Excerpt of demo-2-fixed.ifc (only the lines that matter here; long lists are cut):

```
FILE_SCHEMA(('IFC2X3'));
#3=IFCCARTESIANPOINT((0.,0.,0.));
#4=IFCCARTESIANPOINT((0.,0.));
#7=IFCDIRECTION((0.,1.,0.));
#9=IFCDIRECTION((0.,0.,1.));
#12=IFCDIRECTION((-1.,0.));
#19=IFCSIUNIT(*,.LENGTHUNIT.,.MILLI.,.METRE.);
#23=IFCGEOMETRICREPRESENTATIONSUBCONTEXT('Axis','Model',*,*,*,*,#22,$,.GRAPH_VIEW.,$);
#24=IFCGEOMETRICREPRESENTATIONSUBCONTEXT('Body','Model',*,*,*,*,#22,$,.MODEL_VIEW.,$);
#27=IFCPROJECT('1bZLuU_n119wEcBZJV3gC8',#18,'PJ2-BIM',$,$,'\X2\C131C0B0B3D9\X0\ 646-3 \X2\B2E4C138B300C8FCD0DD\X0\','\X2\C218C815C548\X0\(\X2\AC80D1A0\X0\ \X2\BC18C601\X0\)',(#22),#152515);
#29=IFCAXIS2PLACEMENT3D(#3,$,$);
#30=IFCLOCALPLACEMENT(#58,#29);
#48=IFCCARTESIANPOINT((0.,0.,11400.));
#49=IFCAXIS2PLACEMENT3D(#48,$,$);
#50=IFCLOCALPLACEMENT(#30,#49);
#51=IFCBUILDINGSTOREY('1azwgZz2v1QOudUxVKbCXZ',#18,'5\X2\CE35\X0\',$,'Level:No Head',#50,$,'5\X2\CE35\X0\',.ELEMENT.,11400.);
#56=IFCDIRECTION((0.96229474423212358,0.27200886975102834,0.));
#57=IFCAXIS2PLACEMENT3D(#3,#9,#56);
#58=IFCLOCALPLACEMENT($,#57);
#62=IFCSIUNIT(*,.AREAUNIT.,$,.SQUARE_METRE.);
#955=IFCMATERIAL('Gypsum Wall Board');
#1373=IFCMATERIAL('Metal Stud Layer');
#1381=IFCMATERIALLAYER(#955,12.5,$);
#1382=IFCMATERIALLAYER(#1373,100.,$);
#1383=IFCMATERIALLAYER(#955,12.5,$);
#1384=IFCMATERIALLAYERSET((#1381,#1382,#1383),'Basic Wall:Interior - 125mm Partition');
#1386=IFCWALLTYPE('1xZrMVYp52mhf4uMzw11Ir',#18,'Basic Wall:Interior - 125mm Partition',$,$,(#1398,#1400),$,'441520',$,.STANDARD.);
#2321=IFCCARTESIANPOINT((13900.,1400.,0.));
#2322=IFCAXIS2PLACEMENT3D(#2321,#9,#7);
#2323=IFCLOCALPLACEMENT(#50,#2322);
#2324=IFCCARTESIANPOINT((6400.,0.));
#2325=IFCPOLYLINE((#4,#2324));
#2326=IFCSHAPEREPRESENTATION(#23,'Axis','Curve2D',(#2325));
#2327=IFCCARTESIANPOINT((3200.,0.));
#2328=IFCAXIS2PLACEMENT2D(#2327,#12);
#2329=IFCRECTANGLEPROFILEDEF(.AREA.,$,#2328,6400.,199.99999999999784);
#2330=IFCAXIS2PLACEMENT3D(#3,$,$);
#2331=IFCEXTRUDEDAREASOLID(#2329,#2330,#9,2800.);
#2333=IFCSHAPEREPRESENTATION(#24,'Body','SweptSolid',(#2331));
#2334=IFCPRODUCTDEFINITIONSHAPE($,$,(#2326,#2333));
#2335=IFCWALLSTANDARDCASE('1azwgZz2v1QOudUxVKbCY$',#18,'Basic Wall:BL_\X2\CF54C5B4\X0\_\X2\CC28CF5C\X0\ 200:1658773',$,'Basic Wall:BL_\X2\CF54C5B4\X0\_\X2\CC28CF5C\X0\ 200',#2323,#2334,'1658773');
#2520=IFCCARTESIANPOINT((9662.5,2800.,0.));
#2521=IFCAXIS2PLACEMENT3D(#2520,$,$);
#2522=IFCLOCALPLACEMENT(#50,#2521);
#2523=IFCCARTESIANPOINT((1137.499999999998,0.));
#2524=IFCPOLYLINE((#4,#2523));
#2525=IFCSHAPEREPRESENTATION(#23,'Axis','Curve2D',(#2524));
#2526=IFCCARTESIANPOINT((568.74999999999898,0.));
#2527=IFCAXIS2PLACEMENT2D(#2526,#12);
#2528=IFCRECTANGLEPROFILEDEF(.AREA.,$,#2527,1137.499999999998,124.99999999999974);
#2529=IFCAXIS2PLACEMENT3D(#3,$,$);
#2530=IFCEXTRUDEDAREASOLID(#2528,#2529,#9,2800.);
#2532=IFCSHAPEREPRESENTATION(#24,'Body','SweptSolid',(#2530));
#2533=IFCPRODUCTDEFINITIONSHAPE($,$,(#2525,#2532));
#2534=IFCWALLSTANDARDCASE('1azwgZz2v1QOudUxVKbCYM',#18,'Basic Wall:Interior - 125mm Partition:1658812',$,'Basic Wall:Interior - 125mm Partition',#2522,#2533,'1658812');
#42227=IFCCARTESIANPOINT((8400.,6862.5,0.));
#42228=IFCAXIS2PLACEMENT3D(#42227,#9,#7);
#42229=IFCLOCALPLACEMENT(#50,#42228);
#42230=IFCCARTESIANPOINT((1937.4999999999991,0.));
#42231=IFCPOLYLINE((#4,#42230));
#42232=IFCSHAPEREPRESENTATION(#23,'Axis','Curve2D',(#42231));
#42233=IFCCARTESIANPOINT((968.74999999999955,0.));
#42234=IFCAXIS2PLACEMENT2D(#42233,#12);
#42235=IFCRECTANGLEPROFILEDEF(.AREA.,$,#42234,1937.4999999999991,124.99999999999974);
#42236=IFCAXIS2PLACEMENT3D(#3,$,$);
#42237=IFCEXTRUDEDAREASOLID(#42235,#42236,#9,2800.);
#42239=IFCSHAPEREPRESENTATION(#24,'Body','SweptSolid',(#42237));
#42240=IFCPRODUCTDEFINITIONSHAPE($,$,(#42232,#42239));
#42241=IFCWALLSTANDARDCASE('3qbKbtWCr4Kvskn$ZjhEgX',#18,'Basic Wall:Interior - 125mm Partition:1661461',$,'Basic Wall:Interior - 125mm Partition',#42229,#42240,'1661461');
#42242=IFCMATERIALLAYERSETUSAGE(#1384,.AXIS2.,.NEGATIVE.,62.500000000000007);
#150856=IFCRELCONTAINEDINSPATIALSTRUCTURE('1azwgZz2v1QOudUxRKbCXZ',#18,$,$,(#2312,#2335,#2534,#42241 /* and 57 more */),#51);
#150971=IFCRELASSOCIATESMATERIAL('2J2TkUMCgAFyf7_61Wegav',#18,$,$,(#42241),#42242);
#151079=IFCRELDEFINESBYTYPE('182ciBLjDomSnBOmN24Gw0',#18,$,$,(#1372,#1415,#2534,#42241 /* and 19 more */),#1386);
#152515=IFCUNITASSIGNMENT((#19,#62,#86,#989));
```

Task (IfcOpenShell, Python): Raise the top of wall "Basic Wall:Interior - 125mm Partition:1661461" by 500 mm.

```python
import ifcopenshell
import ifcopenshell.geom
import ifcopenshell.util.representation
import ifcopenshell.util.shape

model = ifcopenshell.open("demo-2-fixed.ifc")
settings = ifcopenshell.geom.settings()


def volume(element):
    """Net volume in cubic metres, openings subtracted."""
    shape = ifcopenshell.geom.create_shape(settings, element)
    return ifcopenshell.util.shape.get_volume(shape.geometry)


wall = model.by_guid("3qbKbtWCr4Kvskn$ZjhEgX")
before = volume(wall)

body = ifcopenshell.util.representation.get_representation(wall, "Model", "Body")
solid = body.Items[0]
old_height = solid.Depth
solid.Depth += 500.0
after = volume(wall)

print(f"height {old_height:g} -> {solid.Depth:g}, volume {before:.3f} -> {after:.3f} m3")

model.write("demo-2-fixed_v2.ifc")
```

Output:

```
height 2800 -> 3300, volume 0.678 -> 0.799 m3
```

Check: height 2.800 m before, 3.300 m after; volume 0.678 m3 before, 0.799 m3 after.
